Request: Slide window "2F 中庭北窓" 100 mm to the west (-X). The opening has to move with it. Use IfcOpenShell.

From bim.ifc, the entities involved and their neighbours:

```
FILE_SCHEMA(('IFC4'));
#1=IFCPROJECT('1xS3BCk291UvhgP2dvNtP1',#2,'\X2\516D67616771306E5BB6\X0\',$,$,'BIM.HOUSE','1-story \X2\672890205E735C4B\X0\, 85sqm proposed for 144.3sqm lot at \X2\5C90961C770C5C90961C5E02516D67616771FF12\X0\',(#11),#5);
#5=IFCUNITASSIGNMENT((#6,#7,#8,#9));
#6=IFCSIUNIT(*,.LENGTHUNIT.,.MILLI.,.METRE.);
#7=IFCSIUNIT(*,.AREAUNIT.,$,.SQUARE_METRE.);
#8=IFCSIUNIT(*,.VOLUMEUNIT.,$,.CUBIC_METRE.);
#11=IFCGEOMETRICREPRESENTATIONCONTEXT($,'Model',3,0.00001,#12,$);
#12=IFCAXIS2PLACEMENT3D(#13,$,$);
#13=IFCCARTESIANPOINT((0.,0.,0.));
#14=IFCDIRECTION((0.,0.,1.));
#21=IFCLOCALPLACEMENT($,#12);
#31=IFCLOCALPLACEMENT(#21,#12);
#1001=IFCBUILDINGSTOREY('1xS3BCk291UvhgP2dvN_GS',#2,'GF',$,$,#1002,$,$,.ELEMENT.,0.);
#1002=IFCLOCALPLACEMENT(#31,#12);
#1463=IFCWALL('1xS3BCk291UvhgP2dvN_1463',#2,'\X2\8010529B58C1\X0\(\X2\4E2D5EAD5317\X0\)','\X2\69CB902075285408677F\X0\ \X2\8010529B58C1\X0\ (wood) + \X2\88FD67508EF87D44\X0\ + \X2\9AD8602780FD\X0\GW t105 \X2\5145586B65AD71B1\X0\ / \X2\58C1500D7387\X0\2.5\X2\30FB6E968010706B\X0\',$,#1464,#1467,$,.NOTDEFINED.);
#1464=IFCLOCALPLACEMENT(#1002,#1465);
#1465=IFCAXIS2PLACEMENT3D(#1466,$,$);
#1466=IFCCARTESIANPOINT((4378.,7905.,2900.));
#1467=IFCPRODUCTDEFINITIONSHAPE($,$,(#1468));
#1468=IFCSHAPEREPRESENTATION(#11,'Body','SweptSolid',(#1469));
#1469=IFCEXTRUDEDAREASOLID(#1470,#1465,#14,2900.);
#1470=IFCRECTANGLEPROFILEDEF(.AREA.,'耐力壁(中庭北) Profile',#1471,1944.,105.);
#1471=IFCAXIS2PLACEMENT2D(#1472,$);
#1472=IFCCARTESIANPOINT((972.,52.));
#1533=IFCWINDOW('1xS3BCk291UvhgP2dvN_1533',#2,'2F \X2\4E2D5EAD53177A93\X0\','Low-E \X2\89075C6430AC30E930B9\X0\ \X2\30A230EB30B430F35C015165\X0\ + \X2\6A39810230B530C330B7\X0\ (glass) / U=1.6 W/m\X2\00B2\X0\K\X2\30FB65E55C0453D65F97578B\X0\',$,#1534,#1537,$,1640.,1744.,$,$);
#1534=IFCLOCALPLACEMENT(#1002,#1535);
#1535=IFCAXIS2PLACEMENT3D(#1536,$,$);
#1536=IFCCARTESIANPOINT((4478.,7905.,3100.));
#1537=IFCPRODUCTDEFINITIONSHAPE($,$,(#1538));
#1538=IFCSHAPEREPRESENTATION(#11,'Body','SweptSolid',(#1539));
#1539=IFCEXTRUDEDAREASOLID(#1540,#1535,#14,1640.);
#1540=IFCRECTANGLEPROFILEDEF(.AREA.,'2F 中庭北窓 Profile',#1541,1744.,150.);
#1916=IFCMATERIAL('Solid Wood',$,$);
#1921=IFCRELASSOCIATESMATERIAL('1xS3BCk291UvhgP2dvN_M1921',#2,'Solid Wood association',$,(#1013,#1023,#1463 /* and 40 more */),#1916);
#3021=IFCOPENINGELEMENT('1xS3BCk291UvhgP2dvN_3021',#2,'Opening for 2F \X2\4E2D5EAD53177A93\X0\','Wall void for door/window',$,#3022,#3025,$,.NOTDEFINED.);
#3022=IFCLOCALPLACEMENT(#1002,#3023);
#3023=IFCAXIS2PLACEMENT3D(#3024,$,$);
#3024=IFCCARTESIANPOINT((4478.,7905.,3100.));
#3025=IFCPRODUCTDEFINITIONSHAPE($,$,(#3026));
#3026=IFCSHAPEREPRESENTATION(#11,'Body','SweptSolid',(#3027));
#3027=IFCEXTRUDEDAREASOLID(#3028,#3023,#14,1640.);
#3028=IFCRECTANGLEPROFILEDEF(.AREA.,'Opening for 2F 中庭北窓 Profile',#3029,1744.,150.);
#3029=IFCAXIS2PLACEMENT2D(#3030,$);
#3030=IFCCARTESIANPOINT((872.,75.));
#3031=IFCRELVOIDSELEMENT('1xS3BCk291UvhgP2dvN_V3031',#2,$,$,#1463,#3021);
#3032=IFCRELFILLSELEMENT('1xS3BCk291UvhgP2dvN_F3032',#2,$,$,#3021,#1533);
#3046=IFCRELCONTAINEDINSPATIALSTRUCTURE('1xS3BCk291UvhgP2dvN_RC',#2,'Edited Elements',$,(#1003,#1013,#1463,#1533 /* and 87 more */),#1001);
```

```python
import ifcopenshell
import ifcopenshell.api.geometry
import ifcopenshell.util.placement

model = ifcopenshell.open("bim.ifc")

window = model.by_guid("1xS3BCk291UvhgP2dvN_1533")
opening = window.FillsVoids[0].RelatingOpeningElement
wall = opening.VoidsElements[0].RelatingBuildingElement

wall_matrix = ifcopenshell.util.placement.get_local_placement(wall.ObjectPlacement)
shift = wall_matrix[:3, 0] * -100.0
before = ifcopenshell.util.placement.get_local_placement(window.ObjectPlacement)[:3, 3].copy()

# The window is not placed relative to its opening, so move both.
for product in (opening, window):
    matrix = ifcopenshell.util.placement.get_local_placement(product.ObjectPlacement)
    matrix[:3, 3] += shift
    ifcopenshell.api.geometry.edit_object_placement(model, product=product, matrix=matrix, is_si=False)

after = ifcopenshell.util.placement.get_local_placement(window.ObjectPlacement)[:3, 3]
print("window moved by", (after - before).round(3) + 0.0)

model.write("bim_v2.ifc")
```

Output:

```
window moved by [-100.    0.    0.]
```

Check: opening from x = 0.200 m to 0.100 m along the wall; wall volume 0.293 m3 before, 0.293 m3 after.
